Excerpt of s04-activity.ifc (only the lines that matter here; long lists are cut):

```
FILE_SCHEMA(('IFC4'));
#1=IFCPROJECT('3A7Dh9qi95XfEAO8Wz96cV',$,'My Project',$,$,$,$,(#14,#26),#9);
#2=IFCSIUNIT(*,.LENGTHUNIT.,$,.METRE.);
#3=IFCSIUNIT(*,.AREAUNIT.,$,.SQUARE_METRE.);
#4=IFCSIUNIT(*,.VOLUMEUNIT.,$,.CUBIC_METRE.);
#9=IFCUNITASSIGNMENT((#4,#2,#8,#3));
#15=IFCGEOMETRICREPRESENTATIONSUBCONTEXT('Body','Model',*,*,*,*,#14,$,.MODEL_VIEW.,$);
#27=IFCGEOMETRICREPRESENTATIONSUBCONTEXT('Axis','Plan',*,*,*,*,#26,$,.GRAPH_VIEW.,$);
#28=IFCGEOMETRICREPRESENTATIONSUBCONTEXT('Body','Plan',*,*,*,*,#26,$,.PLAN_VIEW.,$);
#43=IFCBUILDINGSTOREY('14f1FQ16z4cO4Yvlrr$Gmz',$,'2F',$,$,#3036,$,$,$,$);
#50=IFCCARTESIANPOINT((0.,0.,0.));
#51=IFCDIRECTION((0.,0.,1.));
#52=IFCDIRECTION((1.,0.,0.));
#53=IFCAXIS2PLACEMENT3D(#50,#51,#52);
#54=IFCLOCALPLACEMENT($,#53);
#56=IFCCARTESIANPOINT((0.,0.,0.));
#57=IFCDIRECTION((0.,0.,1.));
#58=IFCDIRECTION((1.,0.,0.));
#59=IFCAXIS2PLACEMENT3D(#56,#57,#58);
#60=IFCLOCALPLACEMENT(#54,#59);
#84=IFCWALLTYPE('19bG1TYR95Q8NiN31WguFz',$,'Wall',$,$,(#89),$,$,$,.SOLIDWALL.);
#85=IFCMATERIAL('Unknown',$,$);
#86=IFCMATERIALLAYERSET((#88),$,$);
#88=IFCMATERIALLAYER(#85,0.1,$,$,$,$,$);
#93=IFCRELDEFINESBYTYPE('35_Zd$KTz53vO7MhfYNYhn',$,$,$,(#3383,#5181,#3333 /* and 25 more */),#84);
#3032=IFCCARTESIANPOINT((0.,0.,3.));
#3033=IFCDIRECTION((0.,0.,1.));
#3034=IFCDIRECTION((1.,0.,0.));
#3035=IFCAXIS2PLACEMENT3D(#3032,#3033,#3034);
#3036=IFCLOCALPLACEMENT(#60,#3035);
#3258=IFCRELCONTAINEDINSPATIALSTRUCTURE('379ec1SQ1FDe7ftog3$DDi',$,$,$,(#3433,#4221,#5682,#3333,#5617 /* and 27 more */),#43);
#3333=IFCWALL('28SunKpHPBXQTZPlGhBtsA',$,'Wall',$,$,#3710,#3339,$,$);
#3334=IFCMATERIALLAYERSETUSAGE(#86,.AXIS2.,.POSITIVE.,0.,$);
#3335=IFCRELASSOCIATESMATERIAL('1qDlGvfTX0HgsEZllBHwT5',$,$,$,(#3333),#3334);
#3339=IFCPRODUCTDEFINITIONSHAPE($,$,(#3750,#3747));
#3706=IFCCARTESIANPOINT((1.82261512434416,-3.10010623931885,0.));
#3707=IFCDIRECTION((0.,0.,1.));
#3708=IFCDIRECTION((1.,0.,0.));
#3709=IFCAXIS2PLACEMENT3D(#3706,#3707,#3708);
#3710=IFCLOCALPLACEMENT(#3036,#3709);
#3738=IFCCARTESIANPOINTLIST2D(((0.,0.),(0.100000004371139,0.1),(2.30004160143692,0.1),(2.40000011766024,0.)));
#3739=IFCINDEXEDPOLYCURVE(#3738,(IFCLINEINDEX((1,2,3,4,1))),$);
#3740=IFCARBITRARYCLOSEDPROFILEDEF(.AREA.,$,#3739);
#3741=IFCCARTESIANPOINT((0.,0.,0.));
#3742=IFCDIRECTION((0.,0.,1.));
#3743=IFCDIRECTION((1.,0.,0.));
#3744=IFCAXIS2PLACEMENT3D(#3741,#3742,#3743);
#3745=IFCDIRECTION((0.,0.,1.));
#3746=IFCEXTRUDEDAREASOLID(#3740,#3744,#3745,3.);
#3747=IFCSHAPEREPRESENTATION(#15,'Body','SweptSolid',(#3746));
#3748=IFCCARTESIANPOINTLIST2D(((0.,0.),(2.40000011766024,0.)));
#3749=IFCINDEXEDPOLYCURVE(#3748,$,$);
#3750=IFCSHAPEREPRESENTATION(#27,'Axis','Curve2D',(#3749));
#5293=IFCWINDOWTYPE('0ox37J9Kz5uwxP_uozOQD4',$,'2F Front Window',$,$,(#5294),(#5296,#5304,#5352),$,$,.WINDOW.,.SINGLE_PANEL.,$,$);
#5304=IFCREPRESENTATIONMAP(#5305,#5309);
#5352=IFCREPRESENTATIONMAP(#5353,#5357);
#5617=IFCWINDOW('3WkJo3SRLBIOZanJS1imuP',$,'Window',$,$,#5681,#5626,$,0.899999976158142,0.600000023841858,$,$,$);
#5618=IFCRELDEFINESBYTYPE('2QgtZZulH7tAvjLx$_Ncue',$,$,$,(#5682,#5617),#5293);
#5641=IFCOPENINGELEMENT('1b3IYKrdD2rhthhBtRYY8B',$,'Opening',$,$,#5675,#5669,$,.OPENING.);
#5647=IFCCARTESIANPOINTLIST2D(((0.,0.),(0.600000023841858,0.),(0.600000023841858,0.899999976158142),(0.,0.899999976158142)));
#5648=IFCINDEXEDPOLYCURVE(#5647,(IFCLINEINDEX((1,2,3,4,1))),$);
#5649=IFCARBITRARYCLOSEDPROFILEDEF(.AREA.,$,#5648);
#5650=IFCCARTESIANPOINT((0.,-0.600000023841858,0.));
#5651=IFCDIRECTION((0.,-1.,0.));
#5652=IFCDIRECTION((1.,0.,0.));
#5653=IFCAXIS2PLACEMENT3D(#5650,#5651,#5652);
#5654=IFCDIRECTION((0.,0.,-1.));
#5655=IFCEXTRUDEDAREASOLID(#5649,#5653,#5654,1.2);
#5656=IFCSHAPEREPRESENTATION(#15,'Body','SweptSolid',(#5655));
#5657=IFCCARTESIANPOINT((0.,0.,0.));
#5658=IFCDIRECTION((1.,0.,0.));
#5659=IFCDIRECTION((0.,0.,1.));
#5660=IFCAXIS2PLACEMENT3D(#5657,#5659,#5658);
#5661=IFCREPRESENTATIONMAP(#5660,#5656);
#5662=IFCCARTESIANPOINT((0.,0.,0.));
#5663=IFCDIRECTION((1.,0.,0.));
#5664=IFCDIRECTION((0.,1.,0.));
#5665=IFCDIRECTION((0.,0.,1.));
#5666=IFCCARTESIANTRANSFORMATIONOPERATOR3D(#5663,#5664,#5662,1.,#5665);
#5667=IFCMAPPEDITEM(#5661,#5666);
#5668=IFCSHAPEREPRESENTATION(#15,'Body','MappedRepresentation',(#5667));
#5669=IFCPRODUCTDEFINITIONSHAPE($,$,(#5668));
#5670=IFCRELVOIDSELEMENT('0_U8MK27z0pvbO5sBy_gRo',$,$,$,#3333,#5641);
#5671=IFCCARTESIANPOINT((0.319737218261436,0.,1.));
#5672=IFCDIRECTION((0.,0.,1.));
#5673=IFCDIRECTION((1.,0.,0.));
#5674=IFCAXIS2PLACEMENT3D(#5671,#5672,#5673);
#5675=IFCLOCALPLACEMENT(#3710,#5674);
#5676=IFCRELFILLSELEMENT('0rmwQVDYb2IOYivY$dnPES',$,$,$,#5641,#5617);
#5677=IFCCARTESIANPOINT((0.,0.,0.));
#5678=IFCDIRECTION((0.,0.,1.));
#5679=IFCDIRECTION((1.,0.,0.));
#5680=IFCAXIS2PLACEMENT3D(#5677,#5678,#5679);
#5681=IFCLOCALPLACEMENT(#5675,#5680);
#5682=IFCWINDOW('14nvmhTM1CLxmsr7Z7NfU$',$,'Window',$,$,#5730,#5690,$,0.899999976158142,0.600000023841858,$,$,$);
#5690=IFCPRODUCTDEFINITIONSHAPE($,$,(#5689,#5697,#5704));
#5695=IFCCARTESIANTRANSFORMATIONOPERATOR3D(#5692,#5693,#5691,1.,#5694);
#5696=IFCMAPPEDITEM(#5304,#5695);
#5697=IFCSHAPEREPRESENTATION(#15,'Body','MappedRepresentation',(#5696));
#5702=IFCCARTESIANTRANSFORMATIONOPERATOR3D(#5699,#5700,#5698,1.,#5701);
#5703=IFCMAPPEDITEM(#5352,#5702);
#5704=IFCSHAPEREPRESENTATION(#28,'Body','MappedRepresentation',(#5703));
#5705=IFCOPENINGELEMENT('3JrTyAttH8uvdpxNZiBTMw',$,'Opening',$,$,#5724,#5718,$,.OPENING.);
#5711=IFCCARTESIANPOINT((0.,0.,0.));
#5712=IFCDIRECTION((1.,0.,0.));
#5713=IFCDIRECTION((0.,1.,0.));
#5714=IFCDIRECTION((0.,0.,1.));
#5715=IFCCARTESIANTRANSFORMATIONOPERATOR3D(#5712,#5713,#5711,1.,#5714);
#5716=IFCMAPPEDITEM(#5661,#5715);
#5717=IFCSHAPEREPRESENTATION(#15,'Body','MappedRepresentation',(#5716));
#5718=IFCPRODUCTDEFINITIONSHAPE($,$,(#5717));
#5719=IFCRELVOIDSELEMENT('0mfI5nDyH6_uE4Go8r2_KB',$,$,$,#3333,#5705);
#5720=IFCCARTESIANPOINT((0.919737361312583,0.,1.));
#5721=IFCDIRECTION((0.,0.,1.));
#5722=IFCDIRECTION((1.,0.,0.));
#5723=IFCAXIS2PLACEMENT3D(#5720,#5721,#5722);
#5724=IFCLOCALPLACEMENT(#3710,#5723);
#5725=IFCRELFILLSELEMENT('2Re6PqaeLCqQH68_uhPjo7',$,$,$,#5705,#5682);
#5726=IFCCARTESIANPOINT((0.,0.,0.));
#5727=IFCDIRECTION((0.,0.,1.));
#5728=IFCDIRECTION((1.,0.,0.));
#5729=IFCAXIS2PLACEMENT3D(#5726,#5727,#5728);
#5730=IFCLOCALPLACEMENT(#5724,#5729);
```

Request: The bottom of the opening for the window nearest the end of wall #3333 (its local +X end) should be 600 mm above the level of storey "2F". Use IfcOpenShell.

```python
import numpy as np
import ifcopenshell
import ifcopenshell.api.geometry
import ifcopenshell.geom
import ifcopenshell.util.element
import ifcopenshell.util.placement
import ifcopenshell.util.shape
import ifcopenshell.util.unit

model = ifcopenshell.open("s04-activity.ifc")
unit_scale = ifcopenshell.util.unit.calculate_unit_scale(model)

window = model.by_guid("14nvmhTM1CLxmsr7Z7NfU$")
opening = window.FillsVoids[0].RelatingOpeningElement
storey = ifcopenshell.util.element.get_container(window, ifc_class="IfcBuildingStorey")
level = ifcopenshell.util.placement.get_local_placement(storey.ObjectPlacement)[2, 3]

# The opening's origin need not be at the sill, so measure its lowest point.
shape = ifcopenshell.geom.create_shape(ifcopenshell.geom.settings(), opening)
bottom = ifcopenshell.util.shape.get_shape_bottom_elevation(shape, shape.geometry) / unit_scale
dz = level + 0.6 / unit_scale - bottom

shift = np.array([0.0, 0.0, dz])
# The window is placed relative to its opening, so it follows when the opening moves.
matrix = ifcopenshell.util.placement.get_local_placement(opening.ObjectPlacement)
matrix[:3, 3] += shift
ifcopenshell.api.geometry.edit_object_placement(
    model, product=opening, matrix=matrix, is_si=False, should_transform_children=True
)

print(f"moved by {dz * unit_scale:+.3f} m")

model.write("s04-activity_updated.ifc")
```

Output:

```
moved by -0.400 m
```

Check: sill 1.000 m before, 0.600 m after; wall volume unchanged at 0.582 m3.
